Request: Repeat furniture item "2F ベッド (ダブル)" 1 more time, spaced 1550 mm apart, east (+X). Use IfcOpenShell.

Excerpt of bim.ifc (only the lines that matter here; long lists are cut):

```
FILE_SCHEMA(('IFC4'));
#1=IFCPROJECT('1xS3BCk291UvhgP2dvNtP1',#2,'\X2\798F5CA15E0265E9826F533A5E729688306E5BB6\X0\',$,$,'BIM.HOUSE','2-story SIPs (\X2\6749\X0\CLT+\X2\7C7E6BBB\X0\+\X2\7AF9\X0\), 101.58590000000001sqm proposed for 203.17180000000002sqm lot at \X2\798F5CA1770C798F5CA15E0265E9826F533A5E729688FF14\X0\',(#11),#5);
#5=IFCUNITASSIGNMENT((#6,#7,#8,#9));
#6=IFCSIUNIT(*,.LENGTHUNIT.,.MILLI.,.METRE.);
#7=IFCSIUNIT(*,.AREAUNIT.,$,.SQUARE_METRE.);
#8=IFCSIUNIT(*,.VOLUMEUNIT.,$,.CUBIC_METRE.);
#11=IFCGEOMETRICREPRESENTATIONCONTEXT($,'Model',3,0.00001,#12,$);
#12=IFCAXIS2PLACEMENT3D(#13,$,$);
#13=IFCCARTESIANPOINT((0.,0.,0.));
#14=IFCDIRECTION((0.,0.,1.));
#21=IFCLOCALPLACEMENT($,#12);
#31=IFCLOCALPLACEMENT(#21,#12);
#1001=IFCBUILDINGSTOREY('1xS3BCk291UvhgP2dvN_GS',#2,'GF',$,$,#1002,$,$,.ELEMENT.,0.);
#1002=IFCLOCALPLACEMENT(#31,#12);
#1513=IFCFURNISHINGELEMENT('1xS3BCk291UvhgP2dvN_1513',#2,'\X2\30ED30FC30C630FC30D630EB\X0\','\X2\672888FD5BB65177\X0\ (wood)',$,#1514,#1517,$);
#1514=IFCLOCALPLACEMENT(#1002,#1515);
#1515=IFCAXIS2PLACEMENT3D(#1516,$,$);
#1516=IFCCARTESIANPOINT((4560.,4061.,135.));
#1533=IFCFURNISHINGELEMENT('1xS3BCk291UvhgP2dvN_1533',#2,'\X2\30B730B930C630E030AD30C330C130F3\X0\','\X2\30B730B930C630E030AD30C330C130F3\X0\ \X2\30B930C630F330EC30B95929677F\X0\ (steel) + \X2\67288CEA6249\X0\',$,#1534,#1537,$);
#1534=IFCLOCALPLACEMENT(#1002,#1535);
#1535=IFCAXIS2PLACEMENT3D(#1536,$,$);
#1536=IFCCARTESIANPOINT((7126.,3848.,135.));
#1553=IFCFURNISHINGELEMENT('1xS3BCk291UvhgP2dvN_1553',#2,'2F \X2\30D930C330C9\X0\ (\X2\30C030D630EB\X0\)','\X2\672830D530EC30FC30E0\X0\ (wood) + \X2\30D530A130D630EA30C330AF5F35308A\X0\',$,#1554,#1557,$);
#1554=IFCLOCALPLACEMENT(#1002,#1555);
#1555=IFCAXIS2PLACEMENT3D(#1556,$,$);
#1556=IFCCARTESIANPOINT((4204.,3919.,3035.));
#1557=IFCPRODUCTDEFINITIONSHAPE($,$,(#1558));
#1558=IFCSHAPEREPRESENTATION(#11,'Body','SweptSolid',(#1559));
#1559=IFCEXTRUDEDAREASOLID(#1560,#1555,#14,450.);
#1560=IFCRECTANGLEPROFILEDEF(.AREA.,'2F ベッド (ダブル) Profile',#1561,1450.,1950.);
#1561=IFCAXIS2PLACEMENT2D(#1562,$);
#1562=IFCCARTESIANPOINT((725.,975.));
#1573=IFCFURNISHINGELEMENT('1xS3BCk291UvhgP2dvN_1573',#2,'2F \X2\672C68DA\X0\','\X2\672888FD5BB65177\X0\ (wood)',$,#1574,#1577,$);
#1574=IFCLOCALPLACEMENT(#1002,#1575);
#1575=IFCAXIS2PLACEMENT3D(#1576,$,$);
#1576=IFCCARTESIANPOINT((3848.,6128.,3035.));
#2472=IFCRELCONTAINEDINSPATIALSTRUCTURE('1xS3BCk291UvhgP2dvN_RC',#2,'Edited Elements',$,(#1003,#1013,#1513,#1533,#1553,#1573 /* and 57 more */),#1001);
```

```python
import numpy as np
import ifcopenshell
import ifcopenshell.api.geometry
import ifcopenshell.api.root
import ifcopenshell.util.element
import ifcopenshell.util.placement

model = ifcopenshell.open("bim.ifc")


def reuse_history(source, copy):
    """copy_class also copies each property set's owner history, people and application; keep the originals."""
    for rel in copy.IsDefinedBy:
        if rel.is_a("IfcRelDefinesByProperties") and (history := rel.RelatingPropertyDefinition.OwnerHistory):
            rel.RelatingPropertyDefinition.OwnerHistory = source.OwnerHistory
            ifcopenshell.util.element.remove_deep2(model, history)


source = model.by_guid("1xS3BCk291UvhgP2dvN_1553")
base = ifcopenshell.util.placement.get_local_placement(source.ObjectPlacement)
step = np.array([1.0, 0.0, 0.0]) * 1550.0

for i in range(1, 2):
    copy = ifcopenshell.api.root.copy_class(model, product=source)
    copy.Representation = ifcopenshell.util.element.copy_deep(
        model, source.Representation, exclude=["IfcGeometricRepresentationContext", "IfcRepresentationMap"]
    )
    reuse_history(source, copy)
    matrix = base.copy()
    matrix[:3, 3] += i * step
    print("added at", matrix[:3, 3].round(3) + 0.0)
    ifcopenshell.api.geometry.edit_object_placement(model, product=copy, matrix=matrix, is_si=False)

model.write("bim-out.ifc")
```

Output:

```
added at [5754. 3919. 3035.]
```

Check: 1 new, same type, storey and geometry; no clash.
